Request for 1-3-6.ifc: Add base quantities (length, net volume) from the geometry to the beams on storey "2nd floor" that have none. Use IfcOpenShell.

First a look at what the model holds.

```python
import ifcopenshell
import ifcopenshell.util.element
import ifcopenshell.util.unit

model = ifcopenshell.open("1-3-6.ifc")
print(model.schema)
for unit_type in ("LENGTHUNIT", "AREAUNIT", "VOLUMEUNIT"):
    print(unit_type, ifcopenshell.util.unit.calculate_unit_scale(model, unit_type))
storey = next(s for s in model.by_type("IfcBuildingStorey") if s.Name == "2nd floor")
beams = [e for e in ifcopenshell.util.element.get_decomposition(storey) if e.is_a("IfcBeam")]
for e in sorted(beams, key=lambda e: e.id()):
    print(e.id(), e.is_a(), e.Name, list(ifcopenshell.util.element.get_psets(e, qtos_only=True)), sep=" | ")
```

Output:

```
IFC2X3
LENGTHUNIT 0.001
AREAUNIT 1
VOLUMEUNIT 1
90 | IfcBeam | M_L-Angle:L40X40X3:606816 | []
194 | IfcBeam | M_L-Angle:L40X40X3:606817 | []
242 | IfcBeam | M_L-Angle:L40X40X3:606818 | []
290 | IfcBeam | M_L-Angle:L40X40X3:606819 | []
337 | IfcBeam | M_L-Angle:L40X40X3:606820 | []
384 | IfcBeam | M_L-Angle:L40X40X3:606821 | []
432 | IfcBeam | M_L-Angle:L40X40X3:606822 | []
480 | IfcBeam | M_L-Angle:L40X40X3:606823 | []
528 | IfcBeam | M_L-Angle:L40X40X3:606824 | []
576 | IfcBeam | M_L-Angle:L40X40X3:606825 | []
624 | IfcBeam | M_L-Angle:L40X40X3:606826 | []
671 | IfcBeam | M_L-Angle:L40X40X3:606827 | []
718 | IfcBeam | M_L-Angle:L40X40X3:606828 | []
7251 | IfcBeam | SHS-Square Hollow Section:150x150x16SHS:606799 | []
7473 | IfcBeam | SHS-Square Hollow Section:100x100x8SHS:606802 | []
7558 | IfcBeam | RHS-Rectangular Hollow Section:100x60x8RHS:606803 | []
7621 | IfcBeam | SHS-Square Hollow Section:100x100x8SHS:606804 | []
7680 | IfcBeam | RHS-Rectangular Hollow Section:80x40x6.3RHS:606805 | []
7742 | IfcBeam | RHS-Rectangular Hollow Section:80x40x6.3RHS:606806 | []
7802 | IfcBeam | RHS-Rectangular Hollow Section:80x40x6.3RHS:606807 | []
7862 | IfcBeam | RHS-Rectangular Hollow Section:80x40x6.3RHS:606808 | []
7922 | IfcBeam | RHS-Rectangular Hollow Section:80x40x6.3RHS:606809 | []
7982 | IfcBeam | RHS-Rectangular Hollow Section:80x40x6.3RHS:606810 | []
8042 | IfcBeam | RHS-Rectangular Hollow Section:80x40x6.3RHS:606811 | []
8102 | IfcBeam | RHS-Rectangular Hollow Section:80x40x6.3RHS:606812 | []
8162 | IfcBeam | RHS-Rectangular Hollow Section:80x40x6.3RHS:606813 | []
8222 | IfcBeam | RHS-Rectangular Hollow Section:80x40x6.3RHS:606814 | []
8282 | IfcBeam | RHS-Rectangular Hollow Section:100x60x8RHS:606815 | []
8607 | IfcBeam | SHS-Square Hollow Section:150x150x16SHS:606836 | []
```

```python
import ifcopenshell
import ifcopenshell.api.pset
import ifcopenshell.geom
import ifcopenshell.util.element
import ifcopenshell.util.shape
import ifcopenshell.util.unit

model = ifcopenshell.open("1-3-6.ifc")
unit_scale = ifcopenshell.util.unit.calculate_unit_scale(model)
volume_scale = ifcopenshell.util.unit.calculate_unit_scale(model, "VOLUMEUNIT")
settings = ifcopenshell.geom.settings()

storey = next(s for s in model.by_type("IfcBuildingStorey") if s.Name == "2nd floor")
beams = [e for e in ifcopenshell.util.element.get_decomposition(storey) if e.is_a("IfcBeam")]

for e in sorted(beams, key=lambda e: e.id()):
    if ifcopenshell.util.element.get_psets(e, qtos_only=True, should_inherit=False):
        continue
    # Geometry comes back in metres, in the element's own axes.
    shape = ifcopenshell.geom.create_shape(settings, e)
    values = {
        "Length": ifcopenshell.util.shape.get_max_xyz(shape.geometry) / unit_scale,
        "NetVolume": ifcopenshell.util.shape.get_volume(shape.geometry) / volume_scale,
    }
    qto = ifcopenshell.api.pset.add_qto(model, product=e, name="BaseQuantities")
    ifcopenshell.api.pset.edit_qto(model, qto=qto, properties=values)
    print(e.id(), {k: round(v, 3) for k, v in values.items()})

model.write("1-3-6_edited.ifc")
```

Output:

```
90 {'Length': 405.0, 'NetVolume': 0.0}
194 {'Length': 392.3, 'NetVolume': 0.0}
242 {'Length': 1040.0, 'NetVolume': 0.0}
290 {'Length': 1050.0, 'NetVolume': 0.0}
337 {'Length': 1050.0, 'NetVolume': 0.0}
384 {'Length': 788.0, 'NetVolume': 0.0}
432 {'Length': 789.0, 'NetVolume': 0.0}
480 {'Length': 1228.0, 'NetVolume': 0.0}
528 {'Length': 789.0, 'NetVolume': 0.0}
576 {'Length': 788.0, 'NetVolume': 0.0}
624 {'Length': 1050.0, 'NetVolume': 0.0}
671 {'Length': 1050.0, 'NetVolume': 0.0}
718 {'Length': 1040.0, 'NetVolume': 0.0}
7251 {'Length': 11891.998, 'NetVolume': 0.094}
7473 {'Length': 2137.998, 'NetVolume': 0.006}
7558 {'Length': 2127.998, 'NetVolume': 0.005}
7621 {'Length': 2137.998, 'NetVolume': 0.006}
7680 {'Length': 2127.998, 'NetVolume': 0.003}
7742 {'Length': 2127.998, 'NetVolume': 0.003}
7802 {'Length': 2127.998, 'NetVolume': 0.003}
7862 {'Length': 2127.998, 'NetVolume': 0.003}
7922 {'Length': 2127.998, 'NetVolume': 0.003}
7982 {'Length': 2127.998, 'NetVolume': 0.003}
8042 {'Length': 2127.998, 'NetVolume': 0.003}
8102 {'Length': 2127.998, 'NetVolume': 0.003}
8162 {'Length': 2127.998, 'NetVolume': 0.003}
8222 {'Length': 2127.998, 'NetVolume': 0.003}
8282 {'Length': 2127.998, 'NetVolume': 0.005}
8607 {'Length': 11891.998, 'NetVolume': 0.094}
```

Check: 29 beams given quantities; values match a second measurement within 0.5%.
